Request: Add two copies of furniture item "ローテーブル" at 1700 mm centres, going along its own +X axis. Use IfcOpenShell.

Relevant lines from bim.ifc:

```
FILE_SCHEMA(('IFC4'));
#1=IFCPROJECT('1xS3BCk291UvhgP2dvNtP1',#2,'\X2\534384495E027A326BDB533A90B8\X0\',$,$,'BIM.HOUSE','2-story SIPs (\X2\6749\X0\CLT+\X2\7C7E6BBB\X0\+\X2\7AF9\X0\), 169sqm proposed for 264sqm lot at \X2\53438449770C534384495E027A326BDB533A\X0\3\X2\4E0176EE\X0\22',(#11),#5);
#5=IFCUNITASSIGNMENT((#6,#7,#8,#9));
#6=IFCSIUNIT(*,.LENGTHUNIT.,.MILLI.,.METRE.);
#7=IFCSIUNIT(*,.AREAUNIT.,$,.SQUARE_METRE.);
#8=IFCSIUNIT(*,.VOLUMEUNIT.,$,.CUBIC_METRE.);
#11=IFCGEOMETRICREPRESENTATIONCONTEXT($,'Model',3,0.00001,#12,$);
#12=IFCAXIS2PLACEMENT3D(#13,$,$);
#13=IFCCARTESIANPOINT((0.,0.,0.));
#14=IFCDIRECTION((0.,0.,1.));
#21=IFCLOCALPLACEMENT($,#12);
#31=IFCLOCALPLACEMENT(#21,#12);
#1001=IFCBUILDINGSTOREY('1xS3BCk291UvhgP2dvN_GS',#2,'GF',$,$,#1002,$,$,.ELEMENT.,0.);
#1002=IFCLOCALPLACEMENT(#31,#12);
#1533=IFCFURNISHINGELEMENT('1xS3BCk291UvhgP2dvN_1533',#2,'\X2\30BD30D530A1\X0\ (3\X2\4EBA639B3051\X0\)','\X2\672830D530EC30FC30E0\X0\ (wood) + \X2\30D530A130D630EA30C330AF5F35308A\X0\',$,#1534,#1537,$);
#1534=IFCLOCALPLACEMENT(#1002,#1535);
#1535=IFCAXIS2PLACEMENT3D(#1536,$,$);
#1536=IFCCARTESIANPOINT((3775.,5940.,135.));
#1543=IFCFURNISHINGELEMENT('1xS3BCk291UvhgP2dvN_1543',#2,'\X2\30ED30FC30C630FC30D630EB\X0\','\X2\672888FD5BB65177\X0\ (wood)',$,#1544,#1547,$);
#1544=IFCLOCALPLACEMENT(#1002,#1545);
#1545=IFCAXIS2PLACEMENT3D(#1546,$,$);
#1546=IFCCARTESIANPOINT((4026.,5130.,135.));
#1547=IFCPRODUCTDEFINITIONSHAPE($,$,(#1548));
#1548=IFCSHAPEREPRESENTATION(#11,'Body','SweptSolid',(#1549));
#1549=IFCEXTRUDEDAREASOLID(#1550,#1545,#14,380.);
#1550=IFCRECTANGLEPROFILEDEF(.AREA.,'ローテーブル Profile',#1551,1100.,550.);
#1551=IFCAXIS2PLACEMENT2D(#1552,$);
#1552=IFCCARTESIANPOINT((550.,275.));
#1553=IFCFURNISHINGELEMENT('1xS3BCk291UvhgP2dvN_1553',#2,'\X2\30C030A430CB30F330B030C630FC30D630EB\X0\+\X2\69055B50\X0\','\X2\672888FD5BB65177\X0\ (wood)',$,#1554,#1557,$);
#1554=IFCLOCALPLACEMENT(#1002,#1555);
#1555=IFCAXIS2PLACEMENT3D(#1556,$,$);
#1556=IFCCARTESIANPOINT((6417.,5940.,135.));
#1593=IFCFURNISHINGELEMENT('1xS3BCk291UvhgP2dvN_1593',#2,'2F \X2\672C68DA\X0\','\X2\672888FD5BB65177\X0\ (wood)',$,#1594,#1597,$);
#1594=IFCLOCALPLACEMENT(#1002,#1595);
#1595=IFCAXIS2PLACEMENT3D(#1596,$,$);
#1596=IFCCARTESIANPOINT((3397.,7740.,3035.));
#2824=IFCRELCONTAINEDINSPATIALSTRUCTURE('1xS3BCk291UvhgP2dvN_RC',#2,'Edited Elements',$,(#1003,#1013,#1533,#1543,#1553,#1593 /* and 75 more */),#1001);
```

```python
import ifcopenshell
import ifcopenshell.api.geometry
import ifcopenshell.api.root
import ifcopenshell.util.element
import ifcopenshell.util.placement
import ifcopenshell.util.unit

model = ifcopenshell.open("bim.ifc")
unit_scale = ifcopenshell.util.unit.calculate_unit_scale(model)


def reuse_history(source, copy):
    """copy_class also copies each property set's owner history, people and application; keep the originals."""
    for rel in copy.IsDefinedBy:
        if rel.is_a("IfcRelDefinesByProperties") and (history := rel.RelatingPropertyDefinition.OwnerHistory):
            rel.RelatingPropertyDefinition.OwnerHistory = source.OwnerHistory
            ifcopenshell.util.element.remove_deep2(model, history)


source = model.by_guid("1xS3BCk291UvhgP2dvN_1543")
base = ifcopenshell.util.placement.get_local_placement(source.ObjectPlacement)
step = base[:3, 0] * 1.7 / unit_scale

for i in range(1, 3):
    copy = ifcopenshell.api.root.copy_class(model, product=source)
    copy.Representation = ifcopenshell.util.element.copy_deep(
        model, source.Representation, exclude=["IfcGeometricRepresentationContext", "IfcRepresentationMap"]
    )
    reuse_history(source, copy)
    matrix = base.copy()
    matrix[:3, 3] += i * step
    print("added at", matrix[:3, 3].round(3) + 0.0)
    ifcopenshell.api.geometry.edit_object_placement(model, product=copy, matrix=matrix, is_si=False)

model.write("bim_rev.ifc")
```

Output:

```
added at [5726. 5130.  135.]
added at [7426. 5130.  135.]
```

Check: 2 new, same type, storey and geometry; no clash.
